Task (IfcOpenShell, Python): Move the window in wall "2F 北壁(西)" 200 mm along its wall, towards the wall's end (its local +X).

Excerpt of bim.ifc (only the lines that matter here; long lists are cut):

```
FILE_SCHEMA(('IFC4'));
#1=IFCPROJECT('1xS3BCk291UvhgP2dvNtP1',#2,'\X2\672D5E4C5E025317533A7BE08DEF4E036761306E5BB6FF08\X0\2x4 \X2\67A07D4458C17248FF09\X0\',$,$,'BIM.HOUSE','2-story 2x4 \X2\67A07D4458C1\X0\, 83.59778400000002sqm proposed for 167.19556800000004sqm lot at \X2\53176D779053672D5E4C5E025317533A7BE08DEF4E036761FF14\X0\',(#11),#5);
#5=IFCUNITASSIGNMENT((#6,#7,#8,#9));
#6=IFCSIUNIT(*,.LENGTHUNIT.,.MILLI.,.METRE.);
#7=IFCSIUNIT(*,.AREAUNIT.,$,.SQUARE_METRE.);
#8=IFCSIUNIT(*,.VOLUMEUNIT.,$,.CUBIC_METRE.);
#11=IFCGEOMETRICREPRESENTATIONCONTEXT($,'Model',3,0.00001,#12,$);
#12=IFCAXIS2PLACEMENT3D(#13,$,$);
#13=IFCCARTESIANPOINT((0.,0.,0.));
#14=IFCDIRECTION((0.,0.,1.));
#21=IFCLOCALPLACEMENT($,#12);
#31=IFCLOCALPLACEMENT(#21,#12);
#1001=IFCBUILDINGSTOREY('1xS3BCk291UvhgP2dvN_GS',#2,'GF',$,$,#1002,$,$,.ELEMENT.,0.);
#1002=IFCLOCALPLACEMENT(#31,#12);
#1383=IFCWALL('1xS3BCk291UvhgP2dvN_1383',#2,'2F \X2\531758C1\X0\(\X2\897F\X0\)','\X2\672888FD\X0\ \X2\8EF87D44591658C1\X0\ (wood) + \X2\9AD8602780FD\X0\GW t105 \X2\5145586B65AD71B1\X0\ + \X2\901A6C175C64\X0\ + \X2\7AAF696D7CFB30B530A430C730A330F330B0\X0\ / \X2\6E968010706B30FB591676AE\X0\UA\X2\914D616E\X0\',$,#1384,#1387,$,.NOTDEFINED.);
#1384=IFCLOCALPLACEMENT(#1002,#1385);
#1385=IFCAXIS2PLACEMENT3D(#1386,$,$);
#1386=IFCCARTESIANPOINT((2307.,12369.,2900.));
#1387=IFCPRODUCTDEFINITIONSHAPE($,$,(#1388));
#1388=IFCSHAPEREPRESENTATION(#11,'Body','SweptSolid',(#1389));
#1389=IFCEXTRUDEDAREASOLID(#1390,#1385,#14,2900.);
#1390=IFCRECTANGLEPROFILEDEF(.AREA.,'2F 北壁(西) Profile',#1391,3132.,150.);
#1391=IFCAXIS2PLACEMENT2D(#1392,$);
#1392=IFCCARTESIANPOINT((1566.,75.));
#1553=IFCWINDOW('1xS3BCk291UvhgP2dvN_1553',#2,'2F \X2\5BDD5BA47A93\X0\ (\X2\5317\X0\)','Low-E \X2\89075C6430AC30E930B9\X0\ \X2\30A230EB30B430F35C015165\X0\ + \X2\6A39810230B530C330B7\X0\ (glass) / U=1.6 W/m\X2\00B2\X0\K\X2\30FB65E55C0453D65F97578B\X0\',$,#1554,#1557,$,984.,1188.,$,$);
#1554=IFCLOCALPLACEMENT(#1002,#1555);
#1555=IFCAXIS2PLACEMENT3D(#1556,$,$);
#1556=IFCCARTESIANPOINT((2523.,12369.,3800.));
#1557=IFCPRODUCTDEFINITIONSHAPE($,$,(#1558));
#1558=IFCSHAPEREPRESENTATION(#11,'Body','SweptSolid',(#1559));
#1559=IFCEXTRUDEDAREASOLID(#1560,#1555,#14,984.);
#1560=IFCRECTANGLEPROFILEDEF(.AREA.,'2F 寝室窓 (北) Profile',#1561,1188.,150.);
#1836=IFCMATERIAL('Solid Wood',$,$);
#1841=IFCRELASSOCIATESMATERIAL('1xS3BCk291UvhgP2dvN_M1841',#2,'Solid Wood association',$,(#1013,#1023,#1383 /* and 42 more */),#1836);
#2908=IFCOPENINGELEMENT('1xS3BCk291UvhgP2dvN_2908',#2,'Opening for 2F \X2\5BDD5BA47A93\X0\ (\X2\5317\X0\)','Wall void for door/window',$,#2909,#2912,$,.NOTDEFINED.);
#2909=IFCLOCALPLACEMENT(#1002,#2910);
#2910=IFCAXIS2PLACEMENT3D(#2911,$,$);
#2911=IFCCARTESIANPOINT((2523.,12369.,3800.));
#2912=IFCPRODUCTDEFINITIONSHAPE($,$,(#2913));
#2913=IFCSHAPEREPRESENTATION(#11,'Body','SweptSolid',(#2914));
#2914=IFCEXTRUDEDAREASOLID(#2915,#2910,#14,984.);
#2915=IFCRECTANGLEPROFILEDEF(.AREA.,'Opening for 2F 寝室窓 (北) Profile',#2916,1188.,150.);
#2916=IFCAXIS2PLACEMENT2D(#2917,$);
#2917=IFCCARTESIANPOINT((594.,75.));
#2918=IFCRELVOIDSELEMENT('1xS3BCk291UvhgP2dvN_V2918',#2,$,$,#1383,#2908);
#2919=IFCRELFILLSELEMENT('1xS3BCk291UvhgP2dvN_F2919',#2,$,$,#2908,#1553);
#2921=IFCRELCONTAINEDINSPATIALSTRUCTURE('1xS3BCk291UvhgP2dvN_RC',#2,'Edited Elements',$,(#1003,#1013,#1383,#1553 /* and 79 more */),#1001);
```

```python
import ifcopenshell
import ifcopenshell.api.geometry
import ifcopenshell.util.placement
import ifcopenshell.util.unit

model = ifcopenshell.open("bim.ifc")
unit_scale = ifcopenshell.util.unit.calculate_unit_scale(model)

window = model.by_id(1553)
opening = window.FillsVoids[0].RelatingOpeningElement
wall = opening.VoidsElements[0].RelatingBuildingElement

wall_matrix = ifcopenshell.util.placement.get_local_placement(wall.ObjectPlacement)
shift = wall_matrix[:3, 0] * 0.2 / unit_scale
before = ifcopenshell.util.placement.get_local_placement(window.ObjectPlacement)[:3, 3].copy()

# The window is not placed relative to its opening, so move both.
for product in (opening, window):
    matrix = ifcopenshell.util.placement.get_local_placement(product.ObjectPlacement)
    matrix[:3, 3] += shift
    ifcopenshell.api.geometry.edit_object_placement(model, product=product, matrix=matrix, is_si=False)

after = ifcopenshell.util.placement.get_local_placement(window.ObjectPlacement)[:3, 3]
print("window moved by", (after - before).round(3) + 0.0)

model.write("bim_updated.ifc")
```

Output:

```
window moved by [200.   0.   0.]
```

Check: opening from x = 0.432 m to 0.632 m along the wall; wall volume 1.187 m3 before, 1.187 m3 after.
